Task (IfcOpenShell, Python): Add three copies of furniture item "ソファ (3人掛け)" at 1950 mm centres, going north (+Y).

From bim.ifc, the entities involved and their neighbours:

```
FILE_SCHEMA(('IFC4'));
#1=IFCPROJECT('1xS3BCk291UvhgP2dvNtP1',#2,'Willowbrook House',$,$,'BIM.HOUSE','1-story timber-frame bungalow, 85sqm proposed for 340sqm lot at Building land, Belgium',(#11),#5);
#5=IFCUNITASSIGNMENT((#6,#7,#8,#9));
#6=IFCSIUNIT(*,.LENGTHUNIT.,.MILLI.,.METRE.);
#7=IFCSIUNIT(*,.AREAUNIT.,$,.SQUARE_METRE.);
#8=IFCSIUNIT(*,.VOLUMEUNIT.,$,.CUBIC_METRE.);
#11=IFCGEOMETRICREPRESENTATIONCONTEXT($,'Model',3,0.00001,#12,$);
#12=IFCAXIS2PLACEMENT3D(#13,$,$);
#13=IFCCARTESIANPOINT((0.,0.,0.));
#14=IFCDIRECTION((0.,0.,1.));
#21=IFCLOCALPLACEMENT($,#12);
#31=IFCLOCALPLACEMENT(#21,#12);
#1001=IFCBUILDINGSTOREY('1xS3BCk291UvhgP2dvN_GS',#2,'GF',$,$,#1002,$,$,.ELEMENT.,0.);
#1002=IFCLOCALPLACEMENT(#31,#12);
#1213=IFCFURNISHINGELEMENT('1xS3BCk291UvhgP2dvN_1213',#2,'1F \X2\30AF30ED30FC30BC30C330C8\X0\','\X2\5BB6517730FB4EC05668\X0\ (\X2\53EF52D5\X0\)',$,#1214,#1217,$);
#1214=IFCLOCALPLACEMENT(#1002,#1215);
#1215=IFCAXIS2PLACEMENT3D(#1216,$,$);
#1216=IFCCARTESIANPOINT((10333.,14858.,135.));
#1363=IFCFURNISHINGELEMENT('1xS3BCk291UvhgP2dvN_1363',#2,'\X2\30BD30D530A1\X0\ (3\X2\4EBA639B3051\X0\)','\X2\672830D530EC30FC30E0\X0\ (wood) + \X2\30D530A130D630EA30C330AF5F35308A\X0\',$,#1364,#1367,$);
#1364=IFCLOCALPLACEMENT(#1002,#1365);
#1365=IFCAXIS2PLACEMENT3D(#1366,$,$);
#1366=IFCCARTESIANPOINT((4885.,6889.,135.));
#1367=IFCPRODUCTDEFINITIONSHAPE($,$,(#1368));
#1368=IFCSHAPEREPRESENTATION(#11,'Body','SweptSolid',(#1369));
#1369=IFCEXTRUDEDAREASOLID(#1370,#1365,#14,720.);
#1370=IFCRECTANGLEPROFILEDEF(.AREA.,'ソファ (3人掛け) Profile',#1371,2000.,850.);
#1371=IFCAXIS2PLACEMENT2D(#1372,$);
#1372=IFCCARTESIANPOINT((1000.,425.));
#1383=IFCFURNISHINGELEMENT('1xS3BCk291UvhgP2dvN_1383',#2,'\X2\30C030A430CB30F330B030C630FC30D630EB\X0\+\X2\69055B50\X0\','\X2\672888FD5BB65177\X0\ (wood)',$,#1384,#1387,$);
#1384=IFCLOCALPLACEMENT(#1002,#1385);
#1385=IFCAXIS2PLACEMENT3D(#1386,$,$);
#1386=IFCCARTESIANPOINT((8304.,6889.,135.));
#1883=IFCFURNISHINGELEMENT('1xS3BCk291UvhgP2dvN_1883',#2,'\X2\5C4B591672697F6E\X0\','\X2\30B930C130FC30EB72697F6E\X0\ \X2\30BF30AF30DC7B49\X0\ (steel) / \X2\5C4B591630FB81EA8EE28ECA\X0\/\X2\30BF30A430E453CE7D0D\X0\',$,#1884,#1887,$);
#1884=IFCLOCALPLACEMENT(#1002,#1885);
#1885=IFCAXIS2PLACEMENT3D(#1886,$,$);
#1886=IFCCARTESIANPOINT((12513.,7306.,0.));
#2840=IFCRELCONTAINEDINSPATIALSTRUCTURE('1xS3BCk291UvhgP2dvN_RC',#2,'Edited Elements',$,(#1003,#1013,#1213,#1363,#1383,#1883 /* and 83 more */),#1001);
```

```python
import numpy as np
import ifcopenshell
import ifcopenshell.api.geometry
import ifcopenshell.api.root
import ifcopenshell.util.element
import ifcopenshell.util.placement
import ifcopenshell.util.unit

model = ifcopenshell.open("bim.ifc")
unit_scale = ifcopenshell.util.unit.calculate_unit_scale(model)


def reuse_history(source, copy):
    """copy_class also copies each property set's owner history, people and application; keep the originals."""
    for rel in copy.IsDefinedBy:
        if rel.is_a("IfcRelDefinesByProperties") and (history := rel.RelatingPropertyDefinition.OwnerHistory):
            rel.RelatingPropertyDefinition.OwnerHistory = source.OwnerHistory
            ifcopenshell.util.element.remove_deep2(model, history)


source = model.by_guid("1xS3BCk291UvhgP2dvN_1363")
base = ifcopenshell.util.placement.get_local_placement(source.ObjectPlacement)
step = np.array([0.0, 1.0, 0.0]) * 1.95 / unit_scale

for i in range(1, 4):
    copy = ifcopenshell.api.root.copy_class(model, product=source)
    copy.Representation = ifcopenshell.util.element.copy_deep(
        model, source.Representation, exclude=["IfcGeometricRepresentationContext", "IfcRepresentationMap"]
    )
    reuse_history(source, copy)
    matrix = base.copy()
    matrix[:3, 3] += i * step
    print("added at", matrix[:3, 3].round(3) + 0.0)
    ifcopenshell.api.geometry.edit_object_placement(model, product=copy, matrix=matrix, is_si=False)

model.write("bim_rev.ifc")
```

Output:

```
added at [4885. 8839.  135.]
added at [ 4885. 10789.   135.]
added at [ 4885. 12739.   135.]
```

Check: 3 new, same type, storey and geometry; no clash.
